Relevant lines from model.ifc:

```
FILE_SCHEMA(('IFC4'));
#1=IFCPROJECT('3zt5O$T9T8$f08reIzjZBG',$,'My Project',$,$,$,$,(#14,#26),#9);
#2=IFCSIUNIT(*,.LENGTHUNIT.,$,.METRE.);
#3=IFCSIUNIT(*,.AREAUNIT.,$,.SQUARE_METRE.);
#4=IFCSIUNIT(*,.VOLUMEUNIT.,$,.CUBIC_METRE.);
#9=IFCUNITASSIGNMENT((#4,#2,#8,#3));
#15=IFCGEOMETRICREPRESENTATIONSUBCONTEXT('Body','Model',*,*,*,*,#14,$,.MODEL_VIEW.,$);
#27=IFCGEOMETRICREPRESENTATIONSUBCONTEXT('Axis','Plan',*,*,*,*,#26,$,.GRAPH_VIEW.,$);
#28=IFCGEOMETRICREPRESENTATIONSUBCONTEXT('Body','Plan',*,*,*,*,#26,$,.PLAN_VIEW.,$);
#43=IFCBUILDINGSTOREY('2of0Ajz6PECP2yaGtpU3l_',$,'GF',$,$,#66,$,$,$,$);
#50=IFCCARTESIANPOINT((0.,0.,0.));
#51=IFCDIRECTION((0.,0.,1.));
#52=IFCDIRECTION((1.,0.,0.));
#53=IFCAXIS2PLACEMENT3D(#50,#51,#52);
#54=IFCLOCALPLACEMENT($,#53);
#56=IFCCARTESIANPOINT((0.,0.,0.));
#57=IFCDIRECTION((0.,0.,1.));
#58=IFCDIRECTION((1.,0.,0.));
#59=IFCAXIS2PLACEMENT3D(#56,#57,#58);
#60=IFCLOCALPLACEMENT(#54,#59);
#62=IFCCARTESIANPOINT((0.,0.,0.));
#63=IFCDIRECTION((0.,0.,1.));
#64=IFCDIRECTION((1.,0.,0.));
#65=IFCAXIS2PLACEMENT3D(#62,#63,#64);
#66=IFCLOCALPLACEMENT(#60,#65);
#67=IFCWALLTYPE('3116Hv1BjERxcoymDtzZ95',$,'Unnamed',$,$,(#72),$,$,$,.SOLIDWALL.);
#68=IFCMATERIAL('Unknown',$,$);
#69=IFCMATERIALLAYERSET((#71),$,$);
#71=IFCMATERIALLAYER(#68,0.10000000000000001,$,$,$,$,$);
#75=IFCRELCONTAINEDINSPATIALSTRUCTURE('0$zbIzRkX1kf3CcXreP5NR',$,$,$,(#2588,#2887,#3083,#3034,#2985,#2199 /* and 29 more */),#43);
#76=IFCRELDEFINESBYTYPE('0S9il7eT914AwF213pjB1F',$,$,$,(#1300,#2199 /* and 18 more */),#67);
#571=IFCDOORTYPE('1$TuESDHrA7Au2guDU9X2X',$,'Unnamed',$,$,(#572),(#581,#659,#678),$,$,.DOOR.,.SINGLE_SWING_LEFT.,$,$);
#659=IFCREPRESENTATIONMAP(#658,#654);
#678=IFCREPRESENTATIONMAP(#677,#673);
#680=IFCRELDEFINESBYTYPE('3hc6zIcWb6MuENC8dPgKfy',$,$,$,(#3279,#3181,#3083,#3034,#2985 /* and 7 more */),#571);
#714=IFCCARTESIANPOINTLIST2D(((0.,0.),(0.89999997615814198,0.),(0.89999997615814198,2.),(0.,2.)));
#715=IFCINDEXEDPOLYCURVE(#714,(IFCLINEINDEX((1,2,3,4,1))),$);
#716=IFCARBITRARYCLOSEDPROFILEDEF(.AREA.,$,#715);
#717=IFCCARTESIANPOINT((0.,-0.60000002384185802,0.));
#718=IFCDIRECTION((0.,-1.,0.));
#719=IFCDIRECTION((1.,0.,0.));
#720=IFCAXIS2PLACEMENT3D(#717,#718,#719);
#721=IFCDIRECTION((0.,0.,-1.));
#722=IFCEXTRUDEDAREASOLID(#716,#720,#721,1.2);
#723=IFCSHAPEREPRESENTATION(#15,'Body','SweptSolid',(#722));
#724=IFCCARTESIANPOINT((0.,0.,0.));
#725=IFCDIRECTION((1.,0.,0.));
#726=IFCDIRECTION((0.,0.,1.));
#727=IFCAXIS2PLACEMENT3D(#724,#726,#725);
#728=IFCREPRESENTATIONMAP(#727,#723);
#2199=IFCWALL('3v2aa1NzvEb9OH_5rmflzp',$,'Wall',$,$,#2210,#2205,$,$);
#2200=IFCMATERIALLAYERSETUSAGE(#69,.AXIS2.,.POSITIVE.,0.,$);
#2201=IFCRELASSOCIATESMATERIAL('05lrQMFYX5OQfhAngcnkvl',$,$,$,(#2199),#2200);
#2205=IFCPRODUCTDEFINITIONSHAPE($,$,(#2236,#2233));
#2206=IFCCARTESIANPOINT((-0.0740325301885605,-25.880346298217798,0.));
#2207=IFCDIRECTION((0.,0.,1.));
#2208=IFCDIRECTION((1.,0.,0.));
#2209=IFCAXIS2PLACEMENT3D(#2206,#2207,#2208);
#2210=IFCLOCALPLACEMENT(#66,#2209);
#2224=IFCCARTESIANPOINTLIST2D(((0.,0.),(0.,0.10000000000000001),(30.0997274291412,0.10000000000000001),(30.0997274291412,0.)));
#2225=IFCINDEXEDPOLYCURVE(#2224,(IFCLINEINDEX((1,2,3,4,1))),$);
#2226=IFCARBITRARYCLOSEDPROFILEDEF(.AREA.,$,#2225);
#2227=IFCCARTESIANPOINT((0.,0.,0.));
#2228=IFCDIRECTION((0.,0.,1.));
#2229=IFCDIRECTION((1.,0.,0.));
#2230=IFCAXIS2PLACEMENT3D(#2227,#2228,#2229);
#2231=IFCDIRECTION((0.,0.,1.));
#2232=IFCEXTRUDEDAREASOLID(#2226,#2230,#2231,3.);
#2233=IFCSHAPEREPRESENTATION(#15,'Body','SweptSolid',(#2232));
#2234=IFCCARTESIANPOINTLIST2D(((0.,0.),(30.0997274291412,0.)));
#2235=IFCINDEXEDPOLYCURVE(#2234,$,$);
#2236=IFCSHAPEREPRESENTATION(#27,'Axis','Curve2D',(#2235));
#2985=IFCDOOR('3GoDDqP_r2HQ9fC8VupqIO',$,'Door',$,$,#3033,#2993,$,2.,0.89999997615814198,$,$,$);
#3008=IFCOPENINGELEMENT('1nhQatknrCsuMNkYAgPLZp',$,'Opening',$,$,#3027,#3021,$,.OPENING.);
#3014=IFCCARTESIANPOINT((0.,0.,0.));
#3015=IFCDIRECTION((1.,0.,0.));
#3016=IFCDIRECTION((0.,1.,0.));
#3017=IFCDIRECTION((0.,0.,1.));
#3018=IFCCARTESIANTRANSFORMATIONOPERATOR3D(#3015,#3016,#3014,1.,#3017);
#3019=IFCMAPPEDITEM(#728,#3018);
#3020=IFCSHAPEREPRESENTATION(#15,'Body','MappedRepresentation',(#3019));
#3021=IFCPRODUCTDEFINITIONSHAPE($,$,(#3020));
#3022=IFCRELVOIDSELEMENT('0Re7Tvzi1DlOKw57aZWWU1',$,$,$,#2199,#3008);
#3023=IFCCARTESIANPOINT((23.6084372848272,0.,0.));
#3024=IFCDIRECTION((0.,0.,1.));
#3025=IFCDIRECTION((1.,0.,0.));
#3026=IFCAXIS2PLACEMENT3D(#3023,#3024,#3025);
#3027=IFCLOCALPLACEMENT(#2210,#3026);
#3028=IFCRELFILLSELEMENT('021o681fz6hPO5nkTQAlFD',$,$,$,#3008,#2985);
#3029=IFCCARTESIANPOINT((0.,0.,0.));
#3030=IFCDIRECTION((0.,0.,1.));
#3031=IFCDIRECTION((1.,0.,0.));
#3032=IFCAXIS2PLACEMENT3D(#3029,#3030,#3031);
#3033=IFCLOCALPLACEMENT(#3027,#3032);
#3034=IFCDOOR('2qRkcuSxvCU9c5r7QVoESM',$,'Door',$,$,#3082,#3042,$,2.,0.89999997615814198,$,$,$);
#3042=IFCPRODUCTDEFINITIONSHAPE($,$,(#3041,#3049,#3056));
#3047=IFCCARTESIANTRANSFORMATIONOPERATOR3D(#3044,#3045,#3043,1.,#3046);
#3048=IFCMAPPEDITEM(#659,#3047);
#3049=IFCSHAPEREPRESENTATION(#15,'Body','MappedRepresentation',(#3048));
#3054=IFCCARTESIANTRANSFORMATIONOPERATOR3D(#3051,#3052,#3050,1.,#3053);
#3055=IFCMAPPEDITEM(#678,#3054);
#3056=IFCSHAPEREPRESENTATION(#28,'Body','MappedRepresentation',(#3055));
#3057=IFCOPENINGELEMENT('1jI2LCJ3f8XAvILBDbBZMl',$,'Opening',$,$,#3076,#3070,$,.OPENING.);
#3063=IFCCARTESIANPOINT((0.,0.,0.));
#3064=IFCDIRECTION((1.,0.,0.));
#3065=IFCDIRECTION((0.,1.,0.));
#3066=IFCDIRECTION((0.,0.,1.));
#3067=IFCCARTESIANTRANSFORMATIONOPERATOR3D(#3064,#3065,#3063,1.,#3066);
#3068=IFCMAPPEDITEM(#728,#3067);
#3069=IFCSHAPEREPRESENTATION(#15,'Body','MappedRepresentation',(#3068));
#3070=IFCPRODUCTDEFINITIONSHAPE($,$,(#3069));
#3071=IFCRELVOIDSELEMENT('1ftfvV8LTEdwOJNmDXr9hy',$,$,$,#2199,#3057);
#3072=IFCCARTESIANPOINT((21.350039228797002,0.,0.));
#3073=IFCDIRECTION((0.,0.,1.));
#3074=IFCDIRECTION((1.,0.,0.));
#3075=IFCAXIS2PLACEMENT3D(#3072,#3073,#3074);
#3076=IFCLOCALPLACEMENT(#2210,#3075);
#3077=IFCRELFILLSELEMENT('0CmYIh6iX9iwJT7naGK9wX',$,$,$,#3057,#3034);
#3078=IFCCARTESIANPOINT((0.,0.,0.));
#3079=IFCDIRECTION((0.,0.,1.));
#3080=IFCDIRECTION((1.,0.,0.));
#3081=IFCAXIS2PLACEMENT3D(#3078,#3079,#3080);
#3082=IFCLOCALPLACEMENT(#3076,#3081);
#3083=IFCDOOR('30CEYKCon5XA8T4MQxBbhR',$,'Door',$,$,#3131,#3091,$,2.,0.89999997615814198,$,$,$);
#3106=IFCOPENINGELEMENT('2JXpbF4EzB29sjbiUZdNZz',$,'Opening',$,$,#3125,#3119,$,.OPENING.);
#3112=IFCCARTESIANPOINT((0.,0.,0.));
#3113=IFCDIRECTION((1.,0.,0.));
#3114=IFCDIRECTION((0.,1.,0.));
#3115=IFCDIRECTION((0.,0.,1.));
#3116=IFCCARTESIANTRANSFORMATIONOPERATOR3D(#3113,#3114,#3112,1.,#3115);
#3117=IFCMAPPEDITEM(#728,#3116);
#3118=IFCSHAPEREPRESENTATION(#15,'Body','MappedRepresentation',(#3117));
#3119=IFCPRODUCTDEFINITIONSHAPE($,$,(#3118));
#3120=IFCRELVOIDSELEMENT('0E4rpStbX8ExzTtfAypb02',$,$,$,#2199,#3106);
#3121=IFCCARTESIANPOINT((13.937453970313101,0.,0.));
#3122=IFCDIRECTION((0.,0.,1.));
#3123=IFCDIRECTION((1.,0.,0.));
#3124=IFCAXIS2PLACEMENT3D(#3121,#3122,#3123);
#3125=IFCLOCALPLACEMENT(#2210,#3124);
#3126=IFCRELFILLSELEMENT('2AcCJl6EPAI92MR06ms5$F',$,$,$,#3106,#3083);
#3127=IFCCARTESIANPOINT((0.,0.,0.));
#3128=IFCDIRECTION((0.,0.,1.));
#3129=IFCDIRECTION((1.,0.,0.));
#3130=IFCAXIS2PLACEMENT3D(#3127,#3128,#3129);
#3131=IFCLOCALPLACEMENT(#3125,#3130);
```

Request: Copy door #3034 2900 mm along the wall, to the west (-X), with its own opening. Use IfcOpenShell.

```python
import ifcopenshell
import ifcopenshell.api.feature
import ifcopenshell.api.geometry
import ifcopenshell.api.root
import ifcopenshell.geom
import ifcopenshell.util.element
import ifcopenshell.util.placement
import ifcopenshell.util.shape

model = ifcopenshell.open("model.ifc")
settings = ifcopenshell.geom.settings()


def volume(element):
    """Net volume in cubic metres, openings subtracted."""
    shape = ifcopenshell.geom.create_shape(settings, element)
    return ifcopenshell.util.shape.get_volume(shape.geometry)


door = model.by_id(3034)
opening = door.FillsVoids[0].RelatingOpeningElement
wall = opening.VoidsElements[0].RelatingBuildingElement
before = volume(wall)
shift = ifcopenshell.util.placement.get_local_placement(wall.ObjectPlacement)[:3, 0] * -2.9

# copy_class copies the void relationship, type, container and properties, but no geometry.
new_opening = ifcopenshell.api.root.copy_class(model, product=opening)
new_opening.Representation = ifcopenshell.util.element.copy_deep(
    model, opening.Representation, exclude=["IfcGeometricRepresentationContext", "IfcRepresentationMap"]
)
new_door = ifcopenshell.api.root.copy_class(model, product=door)
new_door.Representation = ifcopenshell.util.element.copy_deep(
    model, door.Representation, exclude=["IfcGeometricRepresentationContext", "IfcRepresentationMap"]
)
ifcopenshell.api.feature.add_filling(model, opening=new_opening, element=new_door)

for old, new in ((opening, new_opening), (door, new_door)):
    matrix = ifcopenshell.util.placement.get_local_placement(old.ObjectPlacement)
    matrix[:3, 3] += shift
    ifcopenshell.api.geometry.edit_object_placement(model, product=new, matrix=matrix, is_si=False)

after = volume(wall)

print(f"wall volume {before:.3f} -> {after:.3f} m3")

model.write("model_edited.ifc")
```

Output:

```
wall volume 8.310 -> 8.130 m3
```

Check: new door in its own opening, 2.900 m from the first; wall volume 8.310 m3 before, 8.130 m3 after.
